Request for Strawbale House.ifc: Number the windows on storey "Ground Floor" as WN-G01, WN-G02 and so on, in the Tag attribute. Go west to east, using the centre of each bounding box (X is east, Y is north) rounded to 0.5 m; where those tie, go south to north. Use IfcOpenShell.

First a look at what the model holds.

```python
import ifcopenshell
import ifcopenshell.util.element
import ifcopenshell.util.placement

model = ifcopenshell.open("Strawbale House.ifc")
print(model.schema)
storey = next(s for s in model.by_type("IfcBuildingStorey") if s.Name == "Ground Floor")
windows = [e for e in ifcopenshell.util.element.get_decomposition(storey) if e.is_a("IfcWindow")]
for e in sorted(windows, key=lambda e: e.id()):
    origin = ifcopenshell.util.placement.get_local_placement(e.ObjectPlacement)[:3, 3]
    print(e.id(), e.Tag, e.Name, origin.round(2) + 0.0, sep=" | ")
```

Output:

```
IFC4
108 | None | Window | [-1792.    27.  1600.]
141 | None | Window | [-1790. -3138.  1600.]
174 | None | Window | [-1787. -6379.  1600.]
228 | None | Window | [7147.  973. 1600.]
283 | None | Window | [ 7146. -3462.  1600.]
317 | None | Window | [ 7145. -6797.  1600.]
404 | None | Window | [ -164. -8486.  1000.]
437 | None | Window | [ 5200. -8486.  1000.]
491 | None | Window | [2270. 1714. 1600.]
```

```python
import ifcopenshell
import ifcopenshell.geom
import ifcopenshell.util.element
import ifcopenshell.util.shape

model = ifcopenshell.open("Strawbale House.ifc")
settings = ifcopenshell.geom.settings()
settings.set("use-world-coords", True)


def centre(element):
    shape = ifcopenshell.geom.create_shape(settings, element)
    return ifcopenshell.util.shape.get_bbox_centroid(shape.geometry)


storey = next(s for s in model.by_type("IfcBuildingStorey") if s.Name == "Ground Floor")
windows = [e for e in ifcopenshell.util.element.get_decomposition(storey) if e.is_a("IfcWindow")]

# Insertion points can sit at a corner or the storey origin, so sort by the geometry (in metres).
centres = {e: centre(e) for e in windows}
windows.sort(key=lambda e: (round(centres[e][0] / 0.5), centres[e][1]))

for i, e in enumerate(windows, start=1):
    number = f"WN-G{i:02d}"
    e.Tag = number
    print(e.id(), number)

model.write("Strawbale House_updated.ifc")
```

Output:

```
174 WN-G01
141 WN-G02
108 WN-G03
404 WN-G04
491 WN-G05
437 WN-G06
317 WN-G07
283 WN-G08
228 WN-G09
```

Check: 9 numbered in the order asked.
